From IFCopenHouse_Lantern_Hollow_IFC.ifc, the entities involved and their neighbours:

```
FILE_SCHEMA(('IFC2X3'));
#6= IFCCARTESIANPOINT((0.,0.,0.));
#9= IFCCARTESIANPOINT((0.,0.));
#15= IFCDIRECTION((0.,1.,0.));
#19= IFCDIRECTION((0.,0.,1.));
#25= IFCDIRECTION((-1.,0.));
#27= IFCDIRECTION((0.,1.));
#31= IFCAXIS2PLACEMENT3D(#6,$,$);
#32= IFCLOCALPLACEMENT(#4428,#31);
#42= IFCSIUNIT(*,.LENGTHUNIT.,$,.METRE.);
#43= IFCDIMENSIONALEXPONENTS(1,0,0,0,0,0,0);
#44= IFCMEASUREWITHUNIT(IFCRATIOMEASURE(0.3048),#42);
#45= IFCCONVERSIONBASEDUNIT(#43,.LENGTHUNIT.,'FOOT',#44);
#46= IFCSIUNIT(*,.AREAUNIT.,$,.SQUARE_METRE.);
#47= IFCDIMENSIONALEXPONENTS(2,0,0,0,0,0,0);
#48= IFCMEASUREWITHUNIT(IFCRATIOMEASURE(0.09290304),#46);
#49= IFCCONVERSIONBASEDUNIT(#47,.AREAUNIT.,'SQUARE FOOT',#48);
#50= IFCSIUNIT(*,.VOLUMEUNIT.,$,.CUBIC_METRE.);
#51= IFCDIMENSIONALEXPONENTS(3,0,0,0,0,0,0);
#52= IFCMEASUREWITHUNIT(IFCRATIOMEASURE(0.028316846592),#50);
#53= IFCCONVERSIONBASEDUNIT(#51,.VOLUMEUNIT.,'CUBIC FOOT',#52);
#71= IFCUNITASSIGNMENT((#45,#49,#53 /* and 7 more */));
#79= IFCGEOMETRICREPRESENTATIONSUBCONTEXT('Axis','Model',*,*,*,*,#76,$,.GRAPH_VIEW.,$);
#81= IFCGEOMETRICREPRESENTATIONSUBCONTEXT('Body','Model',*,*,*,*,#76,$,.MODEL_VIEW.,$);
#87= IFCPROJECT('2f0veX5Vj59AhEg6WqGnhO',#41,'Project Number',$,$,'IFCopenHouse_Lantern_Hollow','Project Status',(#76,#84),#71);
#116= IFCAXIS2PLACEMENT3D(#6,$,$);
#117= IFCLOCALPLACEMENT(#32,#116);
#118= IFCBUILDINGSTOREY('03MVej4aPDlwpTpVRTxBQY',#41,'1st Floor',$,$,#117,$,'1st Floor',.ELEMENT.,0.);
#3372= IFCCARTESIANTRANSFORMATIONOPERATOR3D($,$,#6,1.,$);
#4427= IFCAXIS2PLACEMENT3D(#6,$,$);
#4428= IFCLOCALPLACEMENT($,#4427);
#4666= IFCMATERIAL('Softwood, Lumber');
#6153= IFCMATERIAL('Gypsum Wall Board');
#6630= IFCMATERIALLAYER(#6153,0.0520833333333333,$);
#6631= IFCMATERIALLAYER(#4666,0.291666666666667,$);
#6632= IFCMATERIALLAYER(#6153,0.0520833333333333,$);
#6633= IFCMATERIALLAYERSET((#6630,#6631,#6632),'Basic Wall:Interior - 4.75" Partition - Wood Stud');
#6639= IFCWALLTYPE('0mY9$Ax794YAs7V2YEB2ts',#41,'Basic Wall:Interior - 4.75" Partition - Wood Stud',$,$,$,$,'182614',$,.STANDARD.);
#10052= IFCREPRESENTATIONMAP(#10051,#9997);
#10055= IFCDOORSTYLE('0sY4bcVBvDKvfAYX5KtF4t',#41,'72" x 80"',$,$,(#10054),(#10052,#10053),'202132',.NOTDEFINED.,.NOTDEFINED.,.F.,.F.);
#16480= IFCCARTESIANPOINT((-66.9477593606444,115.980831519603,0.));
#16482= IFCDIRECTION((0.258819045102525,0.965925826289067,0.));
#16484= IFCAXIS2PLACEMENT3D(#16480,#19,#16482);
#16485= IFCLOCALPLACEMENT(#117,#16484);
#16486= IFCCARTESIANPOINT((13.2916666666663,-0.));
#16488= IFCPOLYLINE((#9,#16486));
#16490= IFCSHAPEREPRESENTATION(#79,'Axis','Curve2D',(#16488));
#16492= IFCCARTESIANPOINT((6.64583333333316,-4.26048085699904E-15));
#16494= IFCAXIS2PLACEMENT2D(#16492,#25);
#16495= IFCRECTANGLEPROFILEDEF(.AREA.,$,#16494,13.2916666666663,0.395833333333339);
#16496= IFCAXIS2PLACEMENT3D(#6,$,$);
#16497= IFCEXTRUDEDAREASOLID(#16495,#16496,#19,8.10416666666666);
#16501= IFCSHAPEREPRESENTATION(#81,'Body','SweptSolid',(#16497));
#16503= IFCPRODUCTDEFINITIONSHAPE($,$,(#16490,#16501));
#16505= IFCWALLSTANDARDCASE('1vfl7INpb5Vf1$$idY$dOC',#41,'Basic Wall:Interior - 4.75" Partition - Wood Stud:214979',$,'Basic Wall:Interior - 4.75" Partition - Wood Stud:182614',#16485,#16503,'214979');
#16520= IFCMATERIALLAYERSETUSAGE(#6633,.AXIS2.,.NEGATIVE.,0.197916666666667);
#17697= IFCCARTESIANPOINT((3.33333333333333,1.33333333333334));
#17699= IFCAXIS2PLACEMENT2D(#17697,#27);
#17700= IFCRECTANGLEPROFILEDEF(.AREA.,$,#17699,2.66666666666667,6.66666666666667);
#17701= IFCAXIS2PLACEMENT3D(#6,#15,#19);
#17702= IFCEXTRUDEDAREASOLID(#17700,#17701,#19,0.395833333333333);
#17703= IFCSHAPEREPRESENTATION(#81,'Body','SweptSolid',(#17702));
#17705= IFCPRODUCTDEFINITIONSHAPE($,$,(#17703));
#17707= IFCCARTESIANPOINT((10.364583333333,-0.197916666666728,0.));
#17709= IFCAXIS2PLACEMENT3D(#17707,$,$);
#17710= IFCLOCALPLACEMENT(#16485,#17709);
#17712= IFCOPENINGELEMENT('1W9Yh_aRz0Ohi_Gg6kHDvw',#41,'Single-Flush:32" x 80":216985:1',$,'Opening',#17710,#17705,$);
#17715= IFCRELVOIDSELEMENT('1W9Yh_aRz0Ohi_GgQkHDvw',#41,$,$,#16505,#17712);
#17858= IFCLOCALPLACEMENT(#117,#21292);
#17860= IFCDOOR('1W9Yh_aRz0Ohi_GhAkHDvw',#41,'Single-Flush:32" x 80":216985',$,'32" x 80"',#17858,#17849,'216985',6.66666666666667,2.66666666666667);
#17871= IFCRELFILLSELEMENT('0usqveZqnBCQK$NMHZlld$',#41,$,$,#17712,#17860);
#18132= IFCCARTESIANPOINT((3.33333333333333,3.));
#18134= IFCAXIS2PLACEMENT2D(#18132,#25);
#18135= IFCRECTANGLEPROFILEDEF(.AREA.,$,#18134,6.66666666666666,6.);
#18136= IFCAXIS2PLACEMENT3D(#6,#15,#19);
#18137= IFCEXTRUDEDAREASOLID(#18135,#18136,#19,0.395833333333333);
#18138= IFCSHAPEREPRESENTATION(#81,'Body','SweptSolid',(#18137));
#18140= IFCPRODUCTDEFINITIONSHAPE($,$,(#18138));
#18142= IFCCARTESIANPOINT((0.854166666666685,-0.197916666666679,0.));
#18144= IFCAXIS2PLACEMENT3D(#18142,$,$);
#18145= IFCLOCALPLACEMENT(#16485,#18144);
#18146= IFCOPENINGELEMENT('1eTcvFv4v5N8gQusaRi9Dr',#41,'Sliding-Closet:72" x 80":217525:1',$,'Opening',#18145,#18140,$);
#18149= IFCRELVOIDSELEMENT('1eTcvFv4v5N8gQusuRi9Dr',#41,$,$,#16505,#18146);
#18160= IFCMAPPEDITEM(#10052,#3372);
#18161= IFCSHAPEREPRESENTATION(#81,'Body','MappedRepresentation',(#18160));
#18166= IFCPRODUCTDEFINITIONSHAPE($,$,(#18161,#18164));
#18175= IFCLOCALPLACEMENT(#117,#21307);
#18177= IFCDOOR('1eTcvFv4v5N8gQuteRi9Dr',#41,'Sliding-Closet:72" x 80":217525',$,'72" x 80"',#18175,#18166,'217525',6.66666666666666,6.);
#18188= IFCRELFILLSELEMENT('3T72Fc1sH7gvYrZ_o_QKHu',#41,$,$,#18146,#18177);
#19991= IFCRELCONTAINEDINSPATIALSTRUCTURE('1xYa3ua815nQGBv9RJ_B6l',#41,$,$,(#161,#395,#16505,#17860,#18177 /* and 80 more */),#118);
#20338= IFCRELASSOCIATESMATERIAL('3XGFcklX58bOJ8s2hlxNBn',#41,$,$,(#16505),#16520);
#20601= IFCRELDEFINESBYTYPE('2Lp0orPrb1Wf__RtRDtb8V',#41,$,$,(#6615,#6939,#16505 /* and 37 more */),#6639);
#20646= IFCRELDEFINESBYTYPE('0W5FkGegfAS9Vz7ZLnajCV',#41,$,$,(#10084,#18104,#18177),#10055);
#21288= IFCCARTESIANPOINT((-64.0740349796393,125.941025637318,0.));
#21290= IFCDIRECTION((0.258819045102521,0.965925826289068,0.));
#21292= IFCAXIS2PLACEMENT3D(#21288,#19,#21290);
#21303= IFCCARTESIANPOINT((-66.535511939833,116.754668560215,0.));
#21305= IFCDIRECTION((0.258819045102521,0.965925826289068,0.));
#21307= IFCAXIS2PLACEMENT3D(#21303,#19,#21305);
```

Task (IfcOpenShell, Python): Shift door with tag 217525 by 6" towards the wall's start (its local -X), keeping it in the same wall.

```python
import ifcopenshell
import ifcopenshell.api.geometry
import ifcopenshell.util.placement
import ifcopenshell.util.unit

model = ifcopenshell.open("IFCopenHouse_Lantern_Hollow_IFC.ifc")
unit_scale = ifcopenshell.util.unit.calculate_unit_scale(model)

door = model.by_guid("1eTcvFv4v5N8gQuteRi9Dr")
opening = door.FillsVoids[0].RelatingOpeningElement
wall = opening.VoidsElements[0].RelatingBuildingElement

wall_matrix = ifcopenshell.util.placement.get_local_placement(wall.ObjectPlacement)
shift = wall_matrix[:3, 0] * -6 * 0.0254 / unit_scale
before = ifcopenshell.util.placement.get_local_placement(door.ObjectPlacement)[:3, 3].copy()

# The door is not placed relative to its opening, so move both.
for product in (opening, door):
    matrix = ifcopenshell.util.placement.get_local_placement(product.ObjectPlacement)
    matrix[:3, 3] += shift
    ifcopenshell.api.geometry.edit_object_placement(model, product=product, matrix=matrix, is_si=False)

after = ifcopenshell.util.placement.get_local_placement(door.ObjectPlacement)[:3, 3]
print("door moved by", (after - before).round(3) + 0.0)

model.write("IFCopenHouse_Lantern_Hollow_IFC-out.ifc")
```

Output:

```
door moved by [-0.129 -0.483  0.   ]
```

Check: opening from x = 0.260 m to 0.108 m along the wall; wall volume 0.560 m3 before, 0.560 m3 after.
